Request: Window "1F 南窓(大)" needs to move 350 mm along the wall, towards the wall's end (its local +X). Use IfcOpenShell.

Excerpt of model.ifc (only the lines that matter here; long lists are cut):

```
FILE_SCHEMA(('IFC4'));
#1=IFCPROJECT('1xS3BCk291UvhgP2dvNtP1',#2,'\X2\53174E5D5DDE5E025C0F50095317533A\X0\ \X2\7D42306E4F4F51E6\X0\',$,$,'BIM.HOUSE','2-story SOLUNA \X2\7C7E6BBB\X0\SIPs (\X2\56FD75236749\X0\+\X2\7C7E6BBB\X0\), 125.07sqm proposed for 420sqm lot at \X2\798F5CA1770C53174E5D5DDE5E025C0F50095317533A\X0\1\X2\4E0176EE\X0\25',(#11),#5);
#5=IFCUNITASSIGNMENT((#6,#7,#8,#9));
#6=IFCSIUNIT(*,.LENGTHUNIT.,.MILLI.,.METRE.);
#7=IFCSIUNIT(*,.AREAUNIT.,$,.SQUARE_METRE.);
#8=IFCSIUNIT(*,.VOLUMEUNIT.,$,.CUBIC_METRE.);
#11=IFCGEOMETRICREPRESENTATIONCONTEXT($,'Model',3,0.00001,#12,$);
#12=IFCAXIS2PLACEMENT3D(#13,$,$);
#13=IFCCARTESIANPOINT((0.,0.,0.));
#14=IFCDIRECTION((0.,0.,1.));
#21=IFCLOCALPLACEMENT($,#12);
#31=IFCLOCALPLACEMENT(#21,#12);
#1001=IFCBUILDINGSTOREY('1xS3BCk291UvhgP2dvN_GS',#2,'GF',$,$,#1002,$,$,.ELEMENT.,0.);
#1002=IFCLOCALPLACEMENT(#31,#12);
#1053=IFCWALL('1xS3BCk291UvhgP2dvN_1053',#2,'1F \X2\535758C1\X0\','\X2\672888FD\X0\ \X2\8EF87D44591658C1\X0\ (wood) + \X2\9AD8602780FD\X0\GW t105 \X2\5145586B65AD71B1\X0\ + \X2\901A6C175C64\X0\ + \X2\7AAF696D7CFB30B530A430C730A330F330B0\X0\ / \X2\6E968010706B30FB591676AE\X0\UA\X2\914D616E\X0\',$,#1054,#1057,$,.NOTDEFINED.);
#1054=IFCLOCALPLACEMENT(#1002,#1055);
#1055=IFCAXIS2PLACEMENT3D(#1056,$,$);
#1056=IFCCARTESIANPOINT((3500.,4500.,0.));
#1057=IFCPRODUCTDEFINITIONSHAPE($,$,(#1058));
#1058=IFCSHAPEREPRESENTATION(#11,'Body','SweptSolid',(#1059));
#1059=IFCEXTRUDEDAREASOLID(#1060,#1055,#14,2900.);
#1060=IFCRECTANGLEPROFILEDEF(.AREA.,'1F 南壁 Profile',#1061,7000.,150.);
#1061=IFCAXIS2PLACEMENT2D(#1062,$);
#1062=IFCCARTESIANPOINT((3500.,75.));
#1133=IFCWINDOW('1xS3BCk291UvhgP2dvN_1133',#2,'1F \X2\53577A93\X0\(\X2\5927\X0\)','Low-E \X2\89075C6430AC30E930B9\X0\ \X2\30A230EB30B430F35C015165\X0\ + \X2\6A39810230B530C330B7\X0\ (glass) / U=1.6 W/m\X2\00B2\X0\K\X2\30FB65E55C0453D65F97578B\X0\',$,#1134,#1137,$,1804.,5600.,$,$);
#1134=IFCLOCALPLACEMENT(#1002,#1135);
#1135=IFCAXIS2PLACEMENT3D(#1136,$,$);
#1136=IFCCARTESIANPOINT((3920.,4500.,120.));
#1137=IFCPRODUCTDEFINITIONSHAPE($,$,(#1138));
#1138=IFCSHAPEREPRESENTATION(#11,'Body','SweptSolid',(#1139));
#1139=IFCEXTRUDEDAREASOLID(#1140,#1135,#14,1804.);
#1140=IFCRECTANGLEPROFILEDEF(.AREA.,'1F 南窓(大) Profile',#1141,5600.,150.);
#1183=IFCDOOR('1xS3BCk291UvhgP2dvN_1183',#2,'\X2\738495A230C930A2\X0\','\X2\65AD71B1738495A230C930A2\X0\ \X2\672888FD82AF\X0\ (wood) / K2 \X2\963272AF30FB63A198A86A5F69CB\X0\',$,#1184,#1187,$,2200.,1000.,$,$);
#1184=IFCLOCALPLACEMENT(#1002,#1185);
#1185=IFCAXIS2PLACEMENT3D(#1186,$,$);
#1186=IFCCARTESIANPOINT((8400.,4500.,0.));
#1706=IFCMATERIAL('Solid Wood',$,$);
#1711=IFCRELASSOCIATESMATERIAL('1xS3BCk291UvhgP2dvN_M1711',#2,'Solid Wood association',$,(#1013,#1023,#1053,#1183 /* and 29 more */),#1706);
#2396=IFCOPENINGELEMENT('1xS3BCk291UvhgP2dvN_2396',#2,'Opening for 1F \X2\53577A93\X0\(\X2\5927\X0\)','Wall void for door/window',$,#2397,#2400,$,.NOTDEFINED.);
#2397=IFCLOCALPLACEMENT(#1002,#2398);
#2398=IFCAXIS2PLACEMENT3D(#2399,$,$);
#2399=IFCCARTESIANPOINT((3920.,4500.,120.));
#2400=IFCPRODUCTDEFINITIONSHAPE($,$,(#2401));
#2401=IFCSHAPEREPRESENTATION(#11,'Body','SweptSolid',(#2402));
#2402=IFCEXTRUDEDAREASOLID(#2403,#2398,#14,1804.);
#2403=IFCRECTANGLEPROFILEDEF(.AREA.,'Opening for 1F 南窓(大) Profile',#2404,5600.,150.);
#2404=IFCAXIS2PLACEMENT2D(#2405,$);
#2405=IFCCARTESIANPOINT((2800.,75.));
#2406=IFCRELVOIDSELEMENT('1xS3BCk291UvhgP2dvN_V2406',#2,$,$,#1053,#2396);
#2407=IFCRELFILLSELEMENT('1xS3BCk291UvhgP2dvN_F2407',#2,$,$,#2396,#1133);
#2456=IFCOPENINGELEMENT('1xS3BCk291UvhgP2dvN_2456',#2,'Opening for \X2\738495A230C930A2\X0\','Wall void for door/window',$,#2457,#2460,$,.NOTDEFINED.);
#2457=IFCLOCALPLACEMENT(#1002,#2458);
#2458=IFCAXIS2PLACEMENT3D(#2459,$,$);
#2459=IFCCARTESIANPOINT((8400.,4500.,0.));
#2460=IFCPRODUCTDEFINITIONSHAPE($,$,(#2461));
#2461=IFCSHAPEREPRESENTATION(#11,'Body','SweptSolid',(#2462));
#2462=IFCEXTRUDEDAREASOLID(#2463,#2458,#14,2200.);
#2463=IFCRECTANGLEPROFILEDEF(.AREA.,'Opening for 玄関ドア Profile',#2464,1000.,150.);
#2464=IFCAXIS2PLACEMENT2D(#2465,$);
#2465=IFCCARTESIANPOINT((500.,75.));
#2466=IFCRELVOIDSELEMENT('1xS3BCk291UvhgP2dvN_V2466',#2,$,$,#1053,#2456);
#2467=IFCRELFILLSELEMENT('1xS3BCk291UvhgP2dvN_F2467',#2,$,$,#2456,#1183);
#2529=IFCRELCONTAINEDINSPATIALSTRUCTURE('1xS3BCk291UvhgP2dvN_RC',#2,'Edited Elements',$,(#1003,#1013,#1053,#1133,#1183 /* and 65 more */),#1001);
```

```python
import ifcopenshell
import ifcopenshell.api.geometry
import ifcopenshell.util.placement
import ifcopenshell.util.unit

model = ifcopenshell.open("model.ifc")
unit_scale = ifcopenshell.util.unit.calculate_unit_scale(model)

window = model.by_guid("1xS3BCk291UvhgP2dvN_1133")
opening = window.FillsVoids[0].RelatingOpeningElement
wall = opening.VoidsElements[0].RelatingBuildingElement

wall_matrix = ifcopenshell.util.placement.get_local_placement(wall.ObjectPlacement)
shift = wall_matrix[:3, 0] * 0.35 / unit_scale
before = ifcopenshell.util.placement.get_local_placement(window.ObjectPlacement)[:3, 3].copy()

# The window is not placed relative to its opening, so move both.
for product in (opening, window):
    matrix = ifcopenshell.util.placement.get_local_placement(product.ObjectPlacement)
    matrix[:3, 3] += shift
    ifcopenshell.api.geometry.edit_object_placement(model, product=product, matrix=matrix, is_si=False)

after = ifcopenshell.util.placement.get_local_placement(window.ObjectPlacement)[:3, 3]
print("window moved by", (after - before).round(3) + 0.0)

model.write("model_edited.ifc")
```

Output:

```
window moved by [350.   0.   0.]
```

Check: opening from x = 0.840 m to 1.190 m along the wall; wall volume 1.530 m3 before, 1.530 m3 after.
